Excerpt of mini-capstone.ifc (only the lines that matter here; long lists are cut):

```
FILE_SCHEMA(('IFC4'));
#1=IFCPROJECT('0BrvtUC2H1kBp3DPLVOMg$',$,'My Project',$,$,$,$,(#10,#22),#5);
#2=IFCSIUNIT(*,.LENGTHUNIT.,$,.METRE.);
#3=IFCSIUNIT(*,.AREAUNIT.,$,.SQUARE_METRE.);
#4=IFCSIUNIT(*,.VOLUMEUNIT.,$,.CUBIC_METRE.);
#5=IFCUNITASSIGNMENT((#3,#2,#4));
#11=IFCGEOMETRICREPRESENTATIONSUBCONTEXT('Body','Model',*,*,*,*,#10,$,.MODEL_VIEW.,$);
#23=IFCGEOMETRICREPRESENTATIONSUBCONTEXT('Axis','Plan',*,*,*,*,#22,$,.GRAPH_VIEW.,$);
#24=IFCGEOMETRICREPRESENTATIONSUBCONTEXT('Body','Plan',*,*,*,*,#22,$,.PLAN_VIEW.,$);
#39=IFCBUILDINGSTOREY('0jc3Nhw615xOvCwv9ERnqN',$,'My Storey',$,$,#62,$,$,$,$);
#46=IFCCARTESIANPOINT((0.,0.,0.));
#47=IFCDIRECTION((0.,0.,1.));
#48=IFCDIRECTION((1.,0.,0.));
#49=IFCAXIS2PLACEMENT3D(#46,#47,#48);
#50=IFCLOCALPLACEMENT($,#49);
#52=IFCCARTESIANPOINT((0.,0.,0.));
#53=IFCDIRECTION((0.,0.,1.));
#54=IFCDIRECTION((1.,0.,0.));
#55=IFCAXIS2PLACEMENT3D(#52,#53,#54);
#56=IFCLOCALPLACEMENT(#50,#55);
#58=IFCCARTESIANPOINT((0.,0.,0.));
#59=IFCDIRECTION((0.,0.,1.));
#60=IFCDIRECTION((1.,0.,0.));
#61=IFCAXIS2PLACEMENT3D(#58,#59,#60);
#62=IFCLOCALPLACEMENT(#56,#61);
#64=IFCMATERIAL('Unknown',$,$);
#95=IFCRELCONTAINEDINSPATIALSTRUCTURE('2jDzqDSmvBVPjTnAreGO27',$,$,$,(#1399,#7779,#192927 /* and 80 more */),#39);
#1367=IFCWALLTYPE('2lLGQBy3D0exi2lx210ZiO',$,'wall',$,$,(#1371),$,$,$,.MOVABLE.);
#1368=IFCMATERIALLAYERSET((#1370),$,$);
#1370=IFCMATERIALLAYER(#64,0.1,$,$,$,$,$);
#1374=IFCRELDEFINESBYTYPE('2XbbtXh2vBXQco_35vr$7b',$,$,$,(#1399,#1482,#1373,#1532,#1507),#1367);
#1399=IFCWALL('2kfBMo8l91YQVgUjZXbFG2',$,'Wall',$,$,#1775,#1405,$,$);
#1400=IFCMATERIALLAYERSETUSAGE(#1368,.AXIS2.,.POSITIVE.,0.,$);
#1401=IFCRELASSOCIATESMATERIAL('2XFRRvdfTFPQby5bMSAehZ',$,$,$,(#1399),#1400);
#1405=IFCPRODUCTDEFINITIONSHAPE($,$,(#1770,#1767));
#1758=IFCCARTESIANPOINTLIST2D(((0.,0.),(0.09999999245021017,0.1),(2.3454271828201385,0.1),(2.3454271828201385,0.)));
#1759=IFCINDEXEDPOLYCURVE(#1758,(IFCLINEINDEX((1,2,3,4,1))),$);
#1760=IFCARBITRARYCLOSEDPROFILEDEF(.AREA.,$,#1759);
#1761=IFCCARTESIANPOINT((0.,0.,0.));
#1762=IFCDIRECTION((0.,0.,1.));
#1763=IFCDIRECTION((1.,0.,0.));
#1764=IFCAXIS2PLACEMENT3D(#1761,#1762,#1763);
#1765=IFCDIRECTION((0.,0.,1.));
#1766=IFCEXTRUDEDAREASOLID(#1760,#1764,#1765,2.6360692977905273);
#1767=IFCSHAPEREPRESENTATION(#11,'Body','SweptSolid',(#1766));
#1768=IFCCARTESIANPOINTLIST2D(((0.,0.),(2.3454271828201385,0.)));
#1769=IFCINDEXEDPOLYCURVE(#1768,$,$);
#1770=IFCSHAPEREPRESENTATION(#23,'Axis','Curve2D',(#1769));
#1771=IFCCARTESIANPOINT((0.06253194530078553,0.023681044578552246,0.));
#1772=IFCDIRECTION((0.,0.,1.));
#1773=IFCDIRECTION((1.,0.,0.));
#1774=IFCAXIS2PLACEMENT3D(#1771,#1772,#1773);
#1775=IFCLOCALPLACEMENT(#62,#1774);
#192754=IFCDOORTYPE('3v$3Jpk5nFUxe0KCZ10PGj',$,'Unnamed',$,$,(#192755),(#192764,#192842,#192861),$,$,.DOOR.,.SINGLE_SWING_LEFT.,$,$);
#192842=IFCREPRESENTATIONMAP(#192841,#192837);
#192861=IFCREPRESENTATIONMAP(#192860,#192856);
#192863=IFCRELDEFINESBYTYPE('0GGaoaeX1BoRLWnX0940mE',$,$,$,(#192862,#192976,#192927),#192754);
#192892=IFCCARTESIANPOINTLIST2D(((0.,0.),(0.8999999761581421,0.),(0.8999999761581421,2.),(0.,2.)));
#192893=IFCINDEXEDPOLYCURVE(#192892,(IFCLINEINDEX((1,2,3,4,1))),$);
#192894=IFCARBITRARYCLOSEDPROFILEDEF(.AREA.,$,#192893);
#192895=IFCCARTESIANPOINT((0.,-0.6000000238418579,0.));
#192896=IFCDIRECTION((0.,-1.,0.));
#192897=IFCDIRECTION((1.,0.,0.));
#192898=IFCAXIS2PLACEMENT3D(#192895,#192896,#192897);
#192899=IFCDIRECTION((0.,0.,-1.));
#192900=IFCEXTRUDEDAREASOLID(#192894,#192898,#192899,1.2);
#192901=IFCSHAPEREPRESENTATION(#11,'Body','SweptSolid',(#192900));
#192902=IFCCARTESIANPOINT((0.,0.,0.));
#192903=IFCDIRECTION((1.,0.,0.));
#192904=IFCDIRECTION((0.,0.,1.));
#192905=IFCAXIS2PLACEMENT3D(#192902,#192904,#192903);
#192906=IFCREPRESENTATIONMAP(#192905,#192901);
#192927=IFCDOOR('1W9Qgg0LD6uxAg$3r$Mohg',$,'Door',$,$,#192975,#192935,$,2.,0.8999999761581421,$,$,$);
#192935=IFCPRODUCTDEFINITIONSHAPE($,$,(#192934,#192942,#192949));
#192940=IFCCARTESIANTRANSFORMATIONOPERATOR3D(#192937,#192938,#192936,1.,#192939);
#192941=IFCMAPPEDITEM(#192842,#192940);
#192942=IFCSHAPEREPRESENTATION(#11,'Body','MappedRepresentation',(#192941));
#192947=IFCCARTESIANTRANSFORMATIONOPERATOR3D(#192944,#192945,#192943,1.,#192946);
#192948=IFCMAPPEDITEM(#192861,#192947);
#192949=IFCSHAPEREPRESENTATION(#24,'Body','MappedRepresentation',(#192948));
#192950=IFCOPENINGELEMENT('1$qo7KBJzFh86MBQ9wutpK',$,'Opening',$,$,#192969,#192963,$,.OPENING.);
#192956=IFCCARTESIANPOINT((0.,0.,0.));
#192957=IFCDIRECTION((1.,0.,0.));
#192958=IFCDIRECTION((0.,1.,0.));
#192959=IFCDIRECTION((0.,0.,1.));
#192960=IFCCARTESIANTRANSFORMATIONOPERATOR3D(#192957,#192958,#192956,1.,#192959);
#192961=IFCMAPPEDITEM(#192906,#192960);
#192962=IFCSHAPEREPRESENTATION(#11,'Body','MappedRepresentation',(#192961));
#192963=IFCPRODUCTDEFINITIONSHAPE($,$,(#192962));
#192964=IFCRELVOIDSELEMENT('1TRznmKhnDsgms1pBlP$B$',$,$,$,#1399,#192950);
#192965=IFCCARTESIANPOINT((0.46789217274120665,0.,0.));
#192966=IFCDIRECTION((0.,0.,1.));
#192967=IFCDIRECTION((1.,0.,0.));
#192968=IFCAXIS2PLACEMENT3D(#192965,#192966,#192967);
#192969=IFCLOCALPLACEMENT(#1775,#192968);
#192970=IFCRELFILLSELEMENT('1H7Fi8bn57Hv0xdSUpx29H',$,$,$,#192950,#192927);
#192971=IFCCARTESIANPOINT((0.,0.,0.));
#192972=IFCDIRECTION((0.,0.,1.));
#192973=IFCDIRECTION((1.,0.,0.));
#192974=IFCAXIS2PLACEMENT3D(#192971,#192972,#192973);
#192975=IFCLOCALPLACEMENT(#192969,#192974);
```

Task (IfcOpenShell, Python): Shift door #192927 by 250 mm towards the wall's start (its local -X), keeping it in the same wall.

```python
import ifcopenshell
import ifcopenshell.api.geometry
import ifcopenshell.util.placement
import ifcopenshell.util.unit

model = ifcopenshell.open("mini-capstone.ifc")
unit_scale = ifcopenshell.util.unit.calculate_unit_scale(model)

door = model.by_guid("1W9Qgg0LD6uxAg$3r$Mohg")
opening = door.FillsVoids[0].RelatingOpeningElement
wall = opening.VoidsElements[0].RelatingBuildingElement

wall_matrix = ifcopenshell.util.placement.get_local_placement(wall.ObjectPlacement)
shift = wall_matrix[:3, 0] * -0.25 / unit_scale
before = ifcopenshell.util.placement.get_local_placement(door.ObjectPlacement)[:3, 3].copy()

# The door is placed relative to its opening, so it follows when the opening moves.
matrix = ifcopenshell.util.placement.get_local_placement(opening.ObjectPlacement)
matrix[:3, 3] += shift
ifcopenshell.api.geometry.edit_object_placement(
    model, product=opening, matrix=matrix, is_si=False, should_transform_children=True
)

after = ifcopenshell.util.placement.get_local_placement(door.ObjectPlacement)[:3, 3]
print("door moved by", (after - before).round(3) + 0.0)

model.write("mini-capstone_edited.ifc")
```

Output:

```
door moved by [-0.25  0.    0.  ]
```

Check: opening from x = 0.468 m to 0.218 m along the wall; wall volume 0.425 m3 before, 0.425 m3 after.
